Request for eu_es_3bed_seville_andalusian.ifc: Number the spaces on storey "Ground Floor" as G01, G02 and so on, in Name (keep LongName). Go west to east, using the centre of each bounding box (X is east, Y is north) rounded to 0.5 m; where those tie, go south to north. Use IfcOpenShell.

First a look at what the model holds.

```python
import ifcopenshell
import ifcopenshell.util.element
import ifcopenshell.util.placement

model = ifcopenshell.open("eu_es_3bed_seville_andalusian.ifc")
print(model.schema)
storey = next(s for s in model.by_type("IfcBuildingStorey") if s.Name == "Ground Floor")
spaces = [e for e in ifcopenshell.util.element.get_decomposition(storey) if e.is_a("IfcSpace")]
for e in sorted(spaces, key=lambda e: e.id()):
    origin = ifcopenshell.util.placement.get_local_placement(e.ObjectPlacement)[:3, 3]
    print(e.id(), e.Name, e.LongName, origin.round(2) + 0.0, sep=" | ")
```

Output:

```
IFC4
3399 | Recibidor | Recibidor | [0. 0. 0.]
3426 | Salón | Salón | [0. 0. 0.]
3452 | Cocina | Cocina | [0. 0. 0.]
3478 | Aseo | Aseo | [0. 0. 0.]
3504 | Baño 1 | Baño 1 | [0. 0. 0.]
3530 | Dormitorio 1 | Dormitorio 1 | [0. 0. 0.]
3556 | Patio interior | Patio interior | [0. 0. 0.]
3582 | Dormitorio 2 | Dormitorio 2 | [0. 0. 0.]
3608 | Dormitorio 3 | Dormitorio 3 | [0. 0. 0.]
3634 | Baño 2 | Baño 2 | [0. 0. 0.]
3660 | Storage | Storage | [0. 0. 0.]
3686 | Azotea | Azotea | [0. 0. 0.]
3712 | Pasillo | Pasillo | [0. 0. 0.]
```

```python
import ifcopenshell
import ifcopenshell.geom
import ifcopenshell.util.element
import ifcopenshell.util.shape

model = ifcopenshell.open("eu_es_3bed_seville_andalusian.ifc")
settings = ifcopenshell.geom.settings()
settings.set("use-world-coords", True)


def centre(element):
    shape = ifcopenshell.geom.create_shape(settings, element)
    return ifcopenshell.util.shape.get_bbox_centroid(shape.geometry)


storey = next(s for s in model.by_type("IfcBuildingStorey") if s.Name == "Ground Floor")
spaces = [e for e in ifcopenshell.util.element.get_decomposition(storey) if e.is_a("IfcSpace")]

# Insertion points can sit at a corner or the storey origin, so sort by the geometry (in metres).
centres = {e: centre(e) for e in spaces}
spaces.sort(key=lambda e: (round(centres[e][0] / 0.5), centres[e][1]))

for i, e in enumerate(spaces, start=1):
    number = f"G{i:02d}"
    e.Name = number
    print(e.id(), number)

model.write("eu_es_3bed_seville_andalusian-out.ifc")
```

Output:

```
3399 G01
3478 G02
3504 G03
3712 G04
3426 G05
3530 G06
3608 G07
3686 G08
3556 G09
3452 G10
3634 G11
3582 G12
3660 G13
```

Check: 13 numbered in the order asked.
